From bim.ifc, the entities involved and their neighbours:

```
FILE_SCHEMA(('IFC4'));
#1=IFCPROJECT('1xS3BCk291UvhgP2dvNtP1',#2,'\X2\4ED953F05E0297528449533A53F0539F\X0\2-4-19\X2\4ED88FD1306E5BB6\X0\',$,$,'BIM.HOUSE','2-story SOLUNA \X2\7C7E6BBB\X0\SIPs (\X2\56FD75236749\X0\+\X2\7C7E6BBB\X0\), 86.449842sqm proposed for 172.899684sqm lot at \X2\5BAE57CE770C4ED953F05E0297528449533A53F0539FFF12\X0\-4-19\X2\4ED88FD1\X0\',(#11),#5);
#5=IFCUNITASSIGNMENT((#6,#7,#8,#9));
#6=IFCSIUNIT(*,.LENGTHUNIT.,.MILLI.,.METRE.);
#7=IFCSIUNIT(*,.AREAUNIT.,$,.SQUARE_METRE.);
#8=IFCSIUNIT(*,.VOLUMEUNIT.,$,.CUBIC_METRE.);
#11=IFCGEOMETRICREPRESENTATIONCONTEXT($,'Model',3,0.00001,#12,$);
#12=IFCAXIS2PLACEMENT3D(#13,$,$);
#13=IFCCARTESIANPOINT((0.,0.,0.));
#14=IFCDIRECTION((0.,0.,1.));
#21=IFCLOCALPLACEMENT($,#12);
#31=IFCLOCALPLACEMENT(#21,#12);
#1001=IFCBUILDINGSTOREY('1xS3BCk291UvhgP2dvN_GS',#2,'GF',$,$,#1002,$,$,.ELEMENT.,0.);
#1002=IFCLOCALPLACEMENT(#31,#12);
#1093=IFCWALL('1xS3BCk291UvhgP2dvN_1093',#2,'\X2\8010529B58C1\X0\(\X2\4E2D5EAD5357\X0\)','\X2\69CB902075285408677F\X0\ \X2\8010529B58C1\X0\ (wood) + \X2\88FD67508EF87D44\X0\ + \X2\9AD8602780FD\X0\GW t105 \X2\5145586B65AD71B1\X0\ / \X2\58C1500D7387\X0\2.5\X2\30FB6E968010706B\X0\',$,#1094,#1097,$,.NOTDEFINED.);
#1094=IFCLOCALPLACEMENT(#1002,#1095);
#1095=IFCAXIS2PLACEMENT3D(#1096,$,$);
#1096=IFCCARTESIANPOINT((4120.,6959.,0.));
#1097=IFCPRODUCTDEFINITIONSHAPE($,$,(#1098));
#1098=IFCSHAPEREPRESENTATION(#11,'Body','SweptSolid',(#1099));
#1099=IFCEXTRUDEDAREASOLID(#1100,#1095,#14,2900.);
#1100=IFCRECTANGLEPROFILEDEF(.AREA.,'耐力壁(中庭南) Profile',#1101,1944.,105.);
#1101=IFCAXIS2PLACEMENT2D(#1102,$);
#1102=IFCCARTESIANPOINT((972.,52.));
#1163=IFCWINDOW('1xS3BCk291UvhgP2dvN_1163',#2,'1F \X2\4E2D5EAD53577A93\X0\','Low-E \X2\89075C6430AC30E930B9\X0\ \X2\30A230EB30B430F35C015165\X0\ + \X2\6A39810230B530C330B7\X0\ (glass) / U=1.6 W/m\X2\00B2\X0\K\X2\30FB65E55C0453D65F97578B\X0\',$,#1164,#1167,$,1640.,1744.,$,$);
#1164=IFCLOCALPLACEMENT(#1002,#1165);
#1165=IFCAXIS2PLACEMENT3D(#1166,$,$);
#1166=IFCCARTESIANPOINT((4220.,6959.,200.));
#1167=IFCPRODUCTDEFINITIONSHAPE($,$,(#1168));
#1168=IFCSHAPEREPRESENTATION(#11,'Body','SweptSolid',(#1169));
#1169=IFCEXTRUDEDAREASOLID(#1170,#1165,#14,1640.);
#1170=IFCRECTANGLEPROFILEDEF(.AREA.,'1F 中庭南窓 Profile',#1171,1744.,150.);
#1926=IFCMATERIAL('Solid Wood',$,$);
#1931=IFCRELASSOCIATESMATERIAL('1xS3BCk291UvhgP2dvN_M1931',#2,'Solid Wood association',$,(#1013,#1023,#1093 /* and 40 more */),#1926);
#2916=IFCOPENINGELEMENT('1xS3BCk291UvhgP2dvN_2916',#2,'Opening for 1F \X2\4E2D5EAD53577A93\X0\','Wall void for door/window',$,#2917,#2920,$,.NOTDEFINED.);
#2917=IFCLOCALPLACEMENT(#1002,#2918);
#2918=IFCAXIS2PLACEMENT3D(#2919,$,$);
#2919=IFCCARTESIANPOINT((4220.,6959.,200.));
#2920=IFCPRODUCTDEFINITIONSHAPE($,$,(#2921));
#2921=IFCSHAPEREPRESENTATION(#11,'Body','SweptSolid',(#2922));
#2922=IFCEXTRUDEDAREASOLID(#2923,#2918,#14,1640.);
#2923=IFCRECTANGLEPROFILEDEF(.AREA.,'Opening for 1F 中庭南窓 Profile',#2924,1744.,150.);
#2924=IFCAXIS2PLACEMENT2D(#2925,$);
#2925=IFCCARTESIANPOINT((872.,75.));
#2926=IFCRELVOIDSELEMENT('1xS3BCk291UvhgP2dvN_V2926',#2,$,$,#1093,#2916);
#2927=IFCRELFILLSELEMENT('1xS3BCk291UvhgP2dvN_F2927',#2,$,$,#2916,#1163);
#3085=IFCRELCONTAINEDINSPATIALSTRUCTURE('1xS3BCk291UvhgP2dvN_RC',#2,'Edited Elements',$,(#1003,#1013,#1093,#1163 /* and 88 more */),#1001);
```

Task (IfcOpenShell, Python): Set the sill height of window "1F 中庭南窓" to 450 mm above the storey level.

```python
import numpy as np
import ifcopenshell
import ifcopenshell.api.geometry
import ifcopenshell.geom
import ifcopenshell.util.element
import ifcopenshell.util.placement
import ifcopenshell.util.shape
import ifcopenshell.util.unit

model = ifcopenshell.open("bim.ifc")
unit_scale = ifcopenshell.util.unit.calculate_unit_scale(model)

window = model.by_id(1163)
opening = window.FillsVoids[0].RelatingOpeningElement
storey = ifcopenshell.util.element.get_container(window, ifc_class="IfcBuildingStorey")
level = ifcopenshell.util.placement.get_local_placement(storey.ObjectPlacement)[2, 3]

# The opening's origin need not be at the sill, so measure its lowest point.
shape = ifcopenshell.geom.create_shape(ifcopenshell.geom.settings(), opening)
bottom = ifcopenshell.util.shape.get_shape_bottom_elevation(shape, shape.geometry) / unit_scale
dz = level + 0.45 / unit_scale - bottom

shift = np.array([0.0, 0.0, dz])
# The window is not placed relative to its opening, so move both.
for product in (opening, window):
    matrix = ifcopenshell.util.placement.get_local_placement(product.ObjectPlacement)
    matrix[:3, 3] += shift
    ifcopenshell.api.geometry.edit_object_placement(model, product=product, matrix=matrix, is_si=False)

print(f"moved by {dz * unit_scale:+.3f} m")

model.write("bim_rev.ifc")
```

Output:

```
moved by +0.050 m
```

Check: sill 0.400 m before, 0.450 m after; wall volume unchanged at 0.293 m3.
